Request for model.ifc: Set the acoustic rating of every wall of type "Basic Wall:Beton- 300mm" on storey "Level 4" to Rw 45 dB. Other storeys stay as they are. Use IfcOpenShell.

First a look at what the model holds.

```python
import ifcopenshell
import ifcopenshell.util.element

model = ifcopenshell.open("model.ifc")
print(model.schema)
storey = next(s for s in model.by_type("IfcBuildingStorey") if s.Name == "Level 4")
walls = [e for e in ifcopenshell.util.element.get_decomposition(storey) if e.is_a("IfcWall")]
seen = {}
for e in walls:
    element_type = ifcopenshell.util.element.get_type(e)
    key = (element_type.Name if element_type != e and element_type else None, ifcopenshell.util.element.get_pset(e, "Pset_WallCommon", "AcousticRating"))
    seen[key] = seen.get(key, 0) + 1
for (name, value), count in sorted(seen.items(), key=str):
    print(count, "x", name, "|", value)
```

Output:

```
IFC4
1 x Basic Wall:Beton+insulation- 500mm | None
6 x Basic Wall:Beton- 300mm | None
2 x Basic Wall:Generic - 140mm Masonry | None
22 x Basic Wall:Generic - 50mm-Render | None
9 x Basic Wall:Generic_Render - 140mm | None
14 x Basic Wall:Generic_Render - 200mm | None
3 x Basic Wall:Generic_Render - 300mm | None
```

```python
import ifcopenshell
import ifcopenshell.api.pset
import ifcopenshell.util.element

model = ifcopenshell.open("model.ifc")

storey = next(s for s in model.by_type("IfcBuildingStorey") if s.Name == "Level 4")
walls = [e for e in ifcopenshell.util.element.get_decomposition(storey) if e.is_a("IfcWall")]

count = 0
for e in walls:
    element_type = ifcopenshell.util.element.get_type(e)
    if element_type in (None, e) or element_type.Name != "Basic Wall:Beton- 300mm":
        continue
    # add_pset returns the element's existing set when there is one.
    pset = ifcopenshell.api.pset.add_pset(model, product=e, name="Pset_WallCommon")
    ifcopenshell.api.pset.edit_pset(model, pset=pset, properties={"AcousticRating": "Rw 45 dB"})
    count += 1

print(count, "walls updated")

model.write("model_rev.ifc")
```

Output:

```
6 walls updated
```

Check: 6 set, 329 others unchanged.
